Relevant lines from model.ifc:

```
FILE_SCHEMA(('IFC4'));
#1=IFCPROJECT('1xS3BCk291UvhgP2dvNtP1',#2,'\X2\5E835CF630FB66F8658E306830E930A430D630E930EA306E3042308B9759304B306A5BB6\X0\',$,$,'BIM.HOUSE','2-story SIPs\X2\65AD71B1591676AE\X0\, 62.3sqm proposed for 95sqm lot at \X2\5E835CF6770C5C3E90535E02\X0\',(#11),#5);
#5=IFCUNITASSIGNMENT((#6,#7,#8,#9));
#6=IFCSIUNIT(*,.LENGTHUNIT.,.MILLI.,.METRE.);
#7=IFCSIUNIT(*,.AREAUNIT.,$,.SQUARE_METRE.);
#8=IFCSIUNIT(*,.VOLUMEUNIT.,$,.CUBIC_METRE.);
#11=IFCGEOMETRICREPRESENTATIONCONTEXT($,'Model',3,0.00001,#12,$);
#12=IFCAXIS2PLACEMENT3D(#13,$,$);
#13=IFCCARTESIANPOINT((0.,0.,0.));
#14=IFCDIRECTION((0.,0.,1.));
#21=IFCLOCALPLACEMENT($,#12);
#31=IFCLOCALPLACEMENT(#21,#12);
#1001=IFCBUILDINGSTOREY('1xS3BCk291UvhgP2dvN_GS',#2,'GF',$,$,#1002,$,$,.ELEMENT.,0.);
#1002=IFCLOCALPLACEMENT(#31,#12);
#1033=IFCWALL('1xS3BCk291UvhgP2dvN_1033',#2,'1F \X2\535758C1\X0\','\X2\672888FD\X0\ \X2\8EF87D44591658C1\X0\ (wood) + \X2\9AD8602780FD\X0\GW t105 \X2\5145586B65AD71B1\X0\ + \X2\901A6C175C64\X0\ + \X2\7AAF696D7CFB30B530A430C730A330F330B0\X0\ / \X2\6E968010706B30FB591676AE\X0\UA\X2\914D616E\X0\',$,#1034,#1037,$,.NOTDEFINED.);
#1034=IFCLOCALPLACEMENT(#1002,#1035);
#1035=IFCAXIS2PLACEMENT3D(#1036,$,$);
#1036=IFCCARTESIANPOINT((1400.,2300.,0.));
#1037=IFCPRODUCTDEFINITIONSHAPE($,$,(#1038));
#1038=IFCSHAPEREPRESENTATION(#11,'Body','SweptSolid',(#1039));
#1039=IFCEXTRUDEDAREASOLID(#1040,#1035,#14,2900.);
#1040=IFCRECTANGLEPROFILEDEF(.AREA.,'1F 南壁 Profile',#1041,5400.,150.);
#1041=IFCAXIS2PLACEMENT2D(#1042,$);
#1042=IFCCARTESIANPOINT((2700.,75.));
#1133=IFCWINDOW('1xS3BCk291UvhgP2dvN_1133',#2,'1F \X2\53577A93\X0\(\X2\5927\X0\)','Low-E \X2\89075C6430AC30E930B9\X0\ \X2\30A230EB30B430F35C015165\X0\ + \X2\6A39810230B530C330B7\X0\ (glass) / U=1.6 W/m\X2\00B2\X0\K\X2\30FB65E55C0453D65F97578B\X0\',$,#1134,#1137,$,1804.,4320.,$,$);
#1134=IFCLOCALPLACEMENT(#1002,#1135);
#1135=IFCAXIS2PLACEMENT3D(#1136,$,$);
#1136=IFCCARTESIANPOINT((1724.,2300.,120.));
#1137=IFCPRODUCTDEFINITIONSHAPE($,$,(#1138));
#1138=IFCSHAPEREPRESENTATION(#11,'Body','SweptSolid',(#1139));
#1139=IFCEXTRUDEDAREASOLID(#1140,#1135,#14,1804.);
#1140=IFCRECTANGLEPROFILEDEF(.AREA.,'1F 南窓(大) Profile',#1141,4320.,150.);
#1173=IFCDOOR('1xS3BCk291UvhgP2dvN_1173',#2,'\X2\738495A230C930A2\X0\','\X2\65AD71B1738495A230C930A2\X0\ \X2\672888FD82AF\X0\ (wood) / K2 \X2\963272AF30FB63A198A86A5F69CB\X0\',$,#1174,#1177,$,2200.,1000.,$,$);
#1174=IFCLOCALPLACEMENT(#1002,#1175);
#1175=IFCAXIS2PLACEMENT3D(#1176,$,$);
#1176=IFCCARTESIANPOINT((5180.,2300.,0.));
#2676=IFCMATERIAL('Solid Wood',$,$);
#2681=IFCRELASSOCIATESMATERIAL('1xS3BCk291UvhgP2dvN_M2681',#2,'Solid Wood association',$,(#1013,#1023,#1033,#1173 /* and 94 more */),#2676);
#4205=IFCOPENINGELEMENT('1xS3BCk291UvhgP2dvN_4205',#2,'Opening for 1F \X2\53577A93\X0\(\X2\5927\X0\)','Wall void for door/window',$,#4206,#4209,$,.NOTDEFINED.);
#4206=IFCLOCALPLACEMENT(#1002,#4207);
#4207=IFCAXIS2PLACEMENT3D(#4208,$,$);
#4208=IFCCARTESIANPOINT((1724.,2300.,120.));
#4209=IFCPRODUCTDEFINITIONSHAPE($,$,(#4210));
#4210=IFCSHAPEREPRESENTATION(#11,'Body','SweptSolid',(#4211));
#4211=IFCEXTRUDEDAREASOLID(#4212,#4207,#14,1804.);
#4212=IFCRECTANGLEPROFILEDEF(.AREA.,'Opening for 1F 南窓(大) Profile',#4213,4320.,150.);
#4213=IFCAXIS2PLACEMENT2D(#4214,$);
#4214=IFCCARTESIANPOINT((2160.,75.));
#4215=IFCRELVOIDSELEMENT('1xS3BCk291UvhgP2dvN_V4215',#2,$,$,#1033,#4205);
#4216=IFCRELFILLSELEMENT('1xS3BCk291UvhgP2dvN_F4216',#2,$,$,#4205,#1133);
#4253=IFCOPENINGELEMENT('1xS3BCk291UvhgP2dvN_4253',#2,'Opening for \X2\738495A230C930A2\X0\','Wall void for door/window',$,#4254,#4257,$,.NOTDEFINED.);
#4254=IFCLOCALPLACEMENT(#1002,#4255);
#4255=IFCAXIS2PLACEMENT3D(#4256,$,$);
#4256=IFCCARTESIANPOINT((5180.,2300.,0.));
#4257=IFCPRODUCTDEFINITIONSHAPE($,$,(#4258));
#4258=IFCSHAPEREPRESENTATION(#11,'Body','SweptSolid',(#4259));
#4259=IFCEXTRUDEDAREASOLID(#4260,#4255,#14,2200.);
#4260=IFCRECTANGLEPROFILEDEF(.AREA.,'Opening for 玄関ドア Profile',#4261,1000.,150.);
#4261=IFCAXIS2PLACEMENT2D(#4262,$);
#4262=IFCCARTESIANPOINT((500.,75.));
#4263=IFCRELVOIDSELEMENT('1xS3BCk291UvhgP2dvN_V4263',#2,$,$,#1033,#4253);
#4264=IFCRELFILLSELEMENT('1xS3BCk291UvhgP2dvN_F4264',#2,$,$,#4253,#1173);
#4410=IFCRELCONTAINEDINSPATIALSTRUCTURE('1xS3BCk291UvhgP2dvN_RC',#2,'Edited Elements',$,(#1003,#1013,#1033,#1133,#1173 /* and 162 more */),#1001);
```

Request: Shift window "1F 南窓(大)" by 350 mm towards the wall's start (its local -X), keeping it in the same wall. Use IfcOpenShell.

```python
import ifcopenshell
import ifcopenshell.api.geometry
import ifcopenshell.util.placement
import ifcopenshell.util.unit

model = ifcopenshell.open("model.ifc")
unit_scale = ifcopenshell.util.unit.calculate_unit_scale(model)

window = model.by_guid("1xS3BCk291UvhgP2dvN_1133")
opening = window.FillsVoids[0].RelatingOpeningElement
wall = opening.VoidsElements[0].RelatingBuildingElement

wall_matrix = ifcopenshell.util.placement.get_local_placement(wall.ObjectPlacement)
shift = wall_matrix[:3, 0] * -0.35 / unit_scale
before = ifcopenshell.util.placement.get_local_placement(window.ObjectPlacement)[:3, 3].copy()

# The window is not placed relative to its opening, so move both.
for product in (opening, window):
    matrix = ifcopenshell.util.placement.get_local_placement(product.ObjectPlacement)
    matrix[:3, 3] += shift
    ifcopenshell.api.geometry.edit_object_placement(model, product=product, matrix=matrix, is_si=False)

after = ifcopenshell.util.placement.get_local_placement(window.ObjectPlacement)[:3, 3]
print("window moved by", (after - before).round(3) + 0.0)

model.write("model-out.ifc")
```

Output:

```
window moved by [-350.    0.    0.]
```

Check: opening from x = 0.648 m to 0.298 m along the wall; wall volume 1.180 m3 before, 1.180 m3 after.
